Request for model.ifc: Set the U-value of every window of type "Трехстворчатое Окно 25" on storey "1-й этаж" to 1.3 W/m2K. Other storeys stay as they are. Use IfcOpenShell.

First a look at what the model holds.

```python
import ifcopenshell
import ifcopenshell.util.element

model = ifcopenshell.open("model.ifc")
print(model.schema)
storey = next(s for s in model.by_type("IfcBuildingStorey") if s.Name == "1-й этаж")
windows = [e for e in ifcopenshell.util.element.get_decomposition(storey) if e.is_a("IfcWindow")]
seen = {}
for e in windows:
    element_type = ifcopenshell.util.element.get_type(e)
    key = (element_type.Name if element_type != e and element_type else None, ifcopenshell.util.element.get_pset(e, "Pset_WindowCommon", "ThermalTransmittance"))
    seen[key] = seen.get(key, 0) + 1
for (name, value), count in sorted(seen.items(), key=str):
    print(count, "x", name, "|", value)
```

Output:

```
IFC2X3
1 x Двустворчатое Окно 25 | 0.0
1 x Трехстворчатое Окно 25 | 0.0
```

```python
import ifcopenshell
import ifcopenshell.api.pset
import ifcopenshell.util.element

model = ifcopenshell.open("model.ifc")

storey = next(s for s in model.by_type("IfcBuildingStorey") if s.Name == "1-й этаж")
windows = [e for e in ifcopenshell.util.element.get_decomposition(storey) if e.is_a("IfcWindow")]

count = 0
for e in windows:
    element_type = ifcopenshell.util.element.get_type(e)
    if element_type in (None, e) or element_type.Name != "Трехстворчатое Окно 25":
        continue
    # add_pset returns the element's existing set when there is one.
    pset = ifcopenshell.api.pset.add_pset(model, product=e, name="Pset_WindowCommon")
    ifcopenshell.api.pset.edit_pset(model, pset=pset, properties={"ThermalTransmittance": 1.3})
    count += 1

print(count, "windows updated")

model.write("model_updated.ifc")
```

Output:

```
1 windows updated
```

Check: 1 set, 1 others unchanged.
